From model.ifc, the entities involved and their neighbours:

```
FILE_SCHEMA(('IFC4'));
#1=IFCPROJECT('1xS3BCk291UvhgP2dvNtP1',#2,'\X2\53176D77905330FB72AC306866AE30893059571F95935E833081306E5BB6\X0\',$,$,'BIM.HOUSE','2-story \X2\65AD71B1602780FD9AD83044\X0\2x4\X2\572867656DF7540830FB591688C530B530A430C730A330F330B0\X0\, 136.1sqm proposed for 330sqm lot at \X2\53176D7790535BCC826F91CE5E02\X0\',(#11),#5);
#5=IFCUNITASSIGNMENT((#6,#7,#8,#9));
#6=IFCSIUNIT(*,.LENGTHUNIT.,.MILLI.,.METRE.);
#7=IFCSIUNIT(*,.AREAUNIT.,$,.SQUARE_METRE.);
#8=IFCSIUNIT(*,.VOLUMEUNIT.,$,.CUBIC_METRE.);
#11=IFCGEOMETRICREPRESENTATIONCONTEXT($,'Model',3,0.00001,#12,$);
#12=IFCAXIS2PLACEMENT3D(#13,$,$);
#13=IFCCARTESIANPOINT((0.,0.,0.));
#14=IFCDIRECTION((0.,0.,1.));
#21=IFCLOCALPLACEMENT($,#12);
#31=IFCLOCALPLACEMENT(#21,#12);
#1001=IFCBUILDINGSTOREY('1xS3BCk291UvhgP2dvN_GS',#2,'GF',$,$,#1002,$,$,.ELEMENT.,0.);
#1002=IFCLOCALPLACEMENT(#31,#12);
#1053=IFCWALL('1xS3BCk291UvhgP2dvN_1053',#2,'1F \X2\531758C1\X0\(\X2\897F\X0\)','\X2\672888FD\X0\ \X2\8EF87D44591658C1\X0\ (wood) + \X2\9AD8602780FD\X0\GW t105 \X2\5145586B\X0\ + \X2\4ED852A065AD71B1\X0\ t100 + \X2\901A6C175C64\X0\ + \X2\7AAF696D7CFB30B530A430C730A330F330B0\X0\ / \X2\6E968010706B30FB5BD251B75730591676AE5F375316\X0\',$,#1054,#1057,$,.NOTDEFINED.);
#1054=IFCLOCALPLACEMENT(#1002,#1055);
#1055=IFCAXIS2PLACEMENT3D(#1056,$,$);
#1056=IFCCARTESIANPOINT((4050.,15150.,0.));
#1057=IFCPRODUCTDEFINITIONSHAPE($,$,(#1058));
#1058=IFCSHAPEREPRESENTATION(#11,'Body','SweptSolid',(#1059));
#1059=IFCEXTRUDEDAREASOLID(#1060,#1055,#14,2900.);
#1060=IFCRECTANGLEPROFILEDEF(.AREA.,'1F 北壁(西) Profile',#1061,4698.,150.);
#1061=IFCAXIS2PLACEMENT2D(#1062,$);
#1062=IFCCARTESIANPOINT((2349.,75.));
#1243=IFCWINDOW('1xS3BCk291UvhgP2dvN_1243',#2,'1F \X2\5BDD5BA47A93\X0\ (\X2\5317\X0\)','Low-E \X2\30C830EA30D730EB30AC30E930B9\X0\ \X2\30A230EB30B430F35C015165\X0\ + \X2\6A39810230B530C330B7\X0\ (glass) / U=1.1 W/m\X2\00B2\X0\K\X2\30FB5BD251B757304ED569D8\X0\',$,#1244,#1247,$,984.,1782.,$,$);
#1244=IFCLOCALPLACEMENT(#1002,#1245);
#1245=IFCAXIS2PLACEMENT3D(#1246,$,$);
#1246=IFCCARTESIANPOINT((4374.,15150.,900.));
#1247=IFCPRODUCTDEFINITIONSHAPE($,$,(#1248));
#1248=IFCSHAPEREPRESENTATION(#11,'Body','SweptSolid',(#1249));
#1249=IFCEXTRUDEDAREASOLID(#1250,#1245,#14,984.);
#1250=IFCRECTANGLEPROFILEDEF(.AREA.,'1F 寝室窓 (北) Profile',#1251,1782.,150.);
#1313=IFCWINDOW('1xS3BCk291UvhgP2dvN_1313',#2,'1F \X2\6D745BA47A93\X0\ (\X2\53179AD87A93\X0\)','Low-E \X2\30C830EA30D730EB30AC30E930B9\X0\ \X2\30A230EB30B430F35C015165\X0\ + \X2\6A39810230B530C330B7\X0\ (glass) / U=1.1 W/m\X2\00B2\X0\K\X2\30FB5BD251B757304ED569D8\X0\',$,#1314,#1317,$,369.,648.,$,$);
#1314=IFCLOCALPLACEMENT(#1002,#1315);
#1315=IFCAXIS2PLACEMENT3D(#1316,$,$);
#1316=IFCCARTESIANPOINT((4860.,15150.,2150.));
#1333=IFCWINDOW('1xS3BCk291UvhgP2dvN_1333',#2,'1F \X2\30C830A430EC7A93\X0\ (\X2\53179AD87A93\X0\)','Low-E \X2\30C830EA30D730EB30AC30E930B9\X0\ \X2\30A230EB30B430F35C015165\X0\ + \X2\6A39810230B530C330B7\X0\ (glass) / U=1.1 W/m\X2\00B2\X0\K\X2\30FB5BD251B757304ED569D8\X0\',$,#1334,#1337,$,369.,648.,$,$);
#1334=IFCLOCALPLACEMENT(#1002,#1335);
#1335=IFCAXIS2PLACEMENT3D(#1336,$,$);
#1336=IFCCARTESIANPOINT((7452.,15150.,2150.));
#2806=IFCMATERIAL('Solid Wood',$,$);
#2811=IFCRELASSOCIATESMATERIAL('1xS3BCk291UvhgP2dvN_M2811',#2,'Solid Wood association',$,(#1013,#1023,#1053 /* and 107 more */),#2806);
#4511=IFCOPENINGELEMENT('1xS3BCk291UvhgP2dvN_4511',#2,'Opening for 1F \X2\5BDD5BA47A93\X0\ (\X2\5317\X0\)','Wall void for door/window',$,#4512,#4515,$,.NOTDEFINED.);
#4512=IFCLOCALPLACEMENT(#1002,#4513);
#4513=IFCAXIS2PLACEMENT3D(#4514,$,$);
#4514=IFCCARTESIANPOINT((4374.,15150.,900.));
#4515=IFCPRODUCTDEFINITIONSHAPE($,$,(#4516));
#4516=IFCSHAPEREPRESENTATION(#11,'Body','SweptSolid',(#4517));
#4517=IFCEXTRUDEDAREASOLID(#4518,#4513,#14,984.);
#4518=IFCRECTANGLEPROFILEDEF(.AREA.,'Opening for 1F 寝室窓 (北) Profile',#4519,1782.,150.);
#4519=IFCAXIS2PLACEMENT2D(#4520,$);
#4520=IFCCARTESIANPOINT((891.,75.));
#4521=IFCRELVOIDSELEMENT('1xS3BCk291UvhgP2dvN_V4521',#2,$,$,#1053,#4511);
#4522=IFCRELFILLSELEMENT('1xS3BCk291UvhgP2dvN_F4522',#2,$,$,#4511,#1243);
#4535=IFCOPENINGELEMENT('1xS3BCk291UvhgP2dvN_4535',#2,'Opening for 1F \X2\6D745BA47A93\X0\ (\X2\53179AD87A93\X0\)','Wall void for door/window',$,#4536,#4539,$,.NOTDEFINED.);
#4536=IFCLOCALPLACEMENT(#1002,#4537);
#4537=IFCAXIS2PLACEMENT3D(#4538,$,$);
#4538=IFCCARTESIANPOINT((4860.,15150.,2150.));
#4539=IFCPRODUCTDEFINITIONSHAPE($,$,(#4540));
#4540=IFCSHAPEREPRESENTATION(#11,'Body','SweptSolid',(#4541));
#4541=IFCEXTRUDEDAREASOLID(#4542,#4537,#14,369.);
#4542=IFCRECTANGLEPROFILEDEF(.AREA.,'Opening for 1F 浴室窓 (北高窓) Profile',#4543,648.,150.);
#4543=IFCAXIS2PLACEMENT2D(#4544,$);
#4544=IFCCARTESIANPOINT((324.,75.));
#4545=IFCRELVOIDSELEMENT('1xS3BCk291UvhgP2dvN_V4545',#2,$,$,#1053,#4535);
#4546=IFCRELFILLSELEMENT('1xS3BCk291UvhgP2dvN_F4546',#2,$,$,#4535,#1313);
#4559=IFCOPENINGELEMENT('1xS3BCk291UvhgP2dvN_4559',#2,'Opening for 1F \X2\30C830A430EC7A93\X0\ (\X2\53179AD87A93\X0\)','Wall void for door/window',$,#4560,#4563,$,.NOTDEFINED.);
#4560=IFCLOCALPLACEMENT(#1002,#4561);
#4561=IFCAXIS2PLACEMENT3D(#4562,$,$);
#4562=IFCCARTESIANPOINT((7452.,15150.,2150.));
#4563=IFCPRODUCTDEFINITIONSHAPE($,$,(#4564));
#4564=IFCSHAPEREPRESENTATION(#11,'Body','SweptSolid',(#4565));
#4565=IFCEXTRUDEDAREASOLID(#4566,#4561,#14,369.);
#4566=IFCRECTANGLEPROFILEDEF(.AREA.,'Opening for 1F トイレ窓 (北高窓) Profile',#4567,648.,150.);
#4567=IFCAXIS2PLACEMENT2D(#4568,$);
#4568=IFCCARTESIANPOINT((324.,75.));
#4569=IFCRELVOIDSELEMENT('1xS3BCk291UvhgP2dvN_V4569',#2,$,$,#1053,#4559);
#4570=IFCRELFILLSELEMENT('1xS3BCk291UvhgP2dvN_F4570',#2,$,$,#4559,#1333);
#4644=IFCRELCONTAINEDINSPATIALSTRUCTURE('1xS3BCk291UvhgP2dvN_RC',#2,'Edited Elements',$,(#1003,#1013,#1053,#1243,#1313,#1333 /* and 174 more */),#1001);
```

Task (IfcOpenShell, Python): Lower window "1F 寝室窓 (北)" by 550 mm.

```python
import numpy as np
import ifcopenshell
import ifcopenshell.api.geometry
import ifcopenshell.util.placement
import ifcopenshell.util.unit

model = ifcopenshell.open("model.ifc")
unit_scale = ifcopenshell.util.unit.calculate_unit_scale(model)

window = model.by_guid("1xS3BCk291UvhgP2dvN_1243")
opening = window.FillsVoids[0].RelatingOpeningElement
dz = -0.55 / unit_scale

shift = np.array([0.0, 0.0, dz])
# The window is not placed relative to its opening, so move both.
for product in (opening, window):
    matrix = ifcopenshell.util.placement.get_local_placement(product.ObjectPlacement)
    matrix[:3, 3] += shift
    ifcopenshell.api.geometry.edit_object_placement(model, product=product, matrix=matrix, is_si=False)

print(f"moved by {dz * unit_scale:+.3f} m")

model.write("model_updated.ifc")
```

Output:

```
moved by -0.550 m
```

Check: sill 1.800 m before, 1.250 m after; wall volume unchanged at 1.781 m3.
